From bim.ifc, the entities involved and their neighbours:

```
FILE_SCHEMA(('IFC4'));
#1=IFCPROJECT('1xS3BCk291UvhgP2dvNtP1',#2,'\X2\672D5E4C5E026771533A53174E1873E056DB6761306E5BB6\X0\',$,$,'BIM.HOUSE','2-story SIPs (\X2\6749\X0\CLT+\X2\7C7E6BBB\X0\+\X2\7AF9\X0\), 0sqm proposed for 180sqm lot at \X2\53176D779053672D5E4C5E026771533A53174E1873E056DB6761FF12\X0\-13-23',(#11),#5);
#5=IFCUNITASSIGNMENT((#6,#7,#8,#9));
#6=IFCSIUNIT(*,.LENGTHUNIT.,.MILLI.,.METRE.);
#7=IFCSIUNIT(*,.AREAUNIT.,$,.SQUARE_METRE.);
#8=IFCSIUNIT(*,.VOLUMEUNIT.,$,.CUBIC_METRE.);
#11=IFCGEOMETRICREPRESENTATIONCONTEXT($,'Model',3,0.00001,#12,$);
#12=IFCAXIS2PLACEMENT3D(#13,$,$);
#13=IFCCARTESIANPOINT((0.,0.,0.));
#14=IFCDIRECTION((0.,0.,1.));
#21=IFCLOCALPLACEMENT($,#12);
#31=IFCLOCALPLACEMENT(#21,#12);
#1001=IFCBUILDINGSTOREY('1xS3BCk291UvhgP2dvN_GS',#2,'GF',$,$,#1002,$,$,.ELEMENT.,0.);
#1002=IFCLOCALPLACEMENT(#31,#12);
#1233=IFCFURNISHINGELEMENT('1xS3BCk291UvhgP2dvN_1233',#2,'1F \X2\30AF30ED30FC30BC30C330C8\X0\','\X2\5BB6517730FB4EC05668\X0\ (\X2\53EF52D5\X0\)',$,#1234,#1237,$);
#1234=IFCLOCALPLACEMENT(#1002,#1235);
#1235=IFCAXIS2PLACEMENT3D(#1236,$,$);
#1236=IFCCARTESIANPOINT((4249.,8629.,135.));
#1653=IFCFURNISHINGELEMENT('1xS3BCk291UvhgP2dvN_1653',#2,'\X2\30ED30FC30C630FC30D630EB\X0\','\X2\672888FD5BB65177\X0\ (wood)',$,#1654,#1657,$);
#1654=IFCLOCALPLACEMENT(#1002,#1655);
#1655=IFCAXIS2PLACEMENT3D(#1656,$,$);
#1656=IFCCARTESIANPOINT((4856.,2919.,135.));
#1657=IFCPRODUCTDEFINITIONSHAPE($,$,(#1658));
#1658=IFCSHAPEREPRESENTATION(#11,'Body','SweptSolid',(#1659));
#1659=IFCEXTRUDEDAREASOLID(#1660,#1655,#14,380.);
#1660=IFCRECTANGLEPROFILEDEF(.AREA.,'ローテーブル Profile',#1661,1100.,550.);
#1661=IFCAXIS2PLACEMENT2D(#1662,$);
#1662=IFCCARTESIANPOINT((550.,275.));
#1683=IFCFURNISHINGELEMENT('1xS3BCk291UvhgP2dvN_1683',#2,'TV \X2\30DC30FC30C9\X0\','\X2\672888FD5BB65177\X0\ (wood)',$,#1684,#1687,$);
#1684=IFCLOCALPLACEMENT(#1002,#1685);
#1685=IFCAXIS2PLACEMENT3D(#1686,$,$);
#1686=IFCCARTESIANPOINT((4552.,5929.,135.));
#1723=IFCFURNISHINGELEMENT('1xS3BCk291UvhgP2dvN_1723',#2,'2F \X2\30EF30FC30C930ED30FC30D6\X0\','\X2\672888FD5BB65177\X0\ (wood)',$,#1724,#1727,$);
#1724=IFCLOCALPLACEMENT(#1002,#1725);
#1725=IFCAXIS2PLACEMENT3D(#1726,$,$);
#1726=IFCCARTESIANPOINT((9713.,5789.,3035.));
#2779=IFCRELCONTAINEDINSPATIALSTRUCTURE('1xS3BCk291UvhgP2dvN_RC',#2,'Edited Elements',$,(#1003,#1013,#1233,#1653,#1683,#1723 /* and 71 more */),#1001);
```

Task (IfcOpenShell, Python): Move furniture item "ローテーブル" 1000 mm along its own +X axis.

```python
import ifcopenshell
import ifcopenshell.api.geometry
import ifcopenshell.util.placement
import ifcopenshell.util.unit

model = ifcopenshell.open("bim.ifc")
unit_scale = ifcopenshell.util.unit.calculate_unit_scale(model)

item = model.by_guid("1xS3BCk291UvhgP2dvN_1653")
matrix = ifcopenshell.util.placement.get_local_placement(item.ObjectPlacement)
matrix[:3, 3] += matrix[:3, 0] * 1 / unit_scale
ifcopenshell.api.geometry.edit_object_placement(model, product=item, matrix=matrix, is_si=False)

print(ifcopenshell.util.placement.get_local_placement(item.ObjectPlacement).round(3) + 0.0)

model.write("bim_v2.ifc")
```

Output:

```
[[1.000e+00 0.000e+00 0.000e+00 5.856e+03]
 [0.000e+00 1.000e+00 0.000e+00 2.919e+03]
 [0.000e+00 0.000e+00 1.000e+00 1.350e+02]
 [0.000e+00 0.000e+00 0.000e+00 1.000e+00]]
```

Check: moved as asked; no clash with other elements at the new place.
